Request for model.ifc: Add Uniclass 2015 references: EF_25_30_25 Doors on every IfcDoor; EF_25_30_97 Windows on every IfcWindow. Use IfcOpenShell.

First a look at what the model holds.

```python
import ifcopenshell

model = ifcopenshell.open("model.ifc")
print(model.schema)
print("classifications:", [c.Name for c in model.by_type("IfcClassification")])
for ifc_class in ("IfcDoor", "IfcRoof", "IfcStair", "IfcWall", "IfcWindow"):
    print(ifc_class, len(model.by_type(ifc_class)))
```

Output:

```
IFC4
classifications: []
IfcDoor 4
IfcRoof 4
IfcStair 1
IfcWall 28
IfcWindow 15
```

```python
import ifcopenshell
import ifcopenshell.api.classification

model = ifcopenshell.open("model.ifc")

system = ifcopenshell.api.classification.add_classification(model, classification="Uniclass 2015")

codes = {
    "IfcDoor": ("EF_25_30_25", "Doors"),
    "IfcWindow": ("EF_25_30_97", "Windows"),
}
for ifc_class, (code, name) in codes.items():
    products = model.by_type(ifc_class)
    ifcopenshell.api.classification.add_reference(
        model, products=products, classification=system, identification=code, name=name
    )
    print(code, len(products))

model.write("model_rev.ifc")
```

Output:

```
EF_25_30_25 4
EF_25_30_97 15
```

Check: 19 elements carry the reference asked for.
